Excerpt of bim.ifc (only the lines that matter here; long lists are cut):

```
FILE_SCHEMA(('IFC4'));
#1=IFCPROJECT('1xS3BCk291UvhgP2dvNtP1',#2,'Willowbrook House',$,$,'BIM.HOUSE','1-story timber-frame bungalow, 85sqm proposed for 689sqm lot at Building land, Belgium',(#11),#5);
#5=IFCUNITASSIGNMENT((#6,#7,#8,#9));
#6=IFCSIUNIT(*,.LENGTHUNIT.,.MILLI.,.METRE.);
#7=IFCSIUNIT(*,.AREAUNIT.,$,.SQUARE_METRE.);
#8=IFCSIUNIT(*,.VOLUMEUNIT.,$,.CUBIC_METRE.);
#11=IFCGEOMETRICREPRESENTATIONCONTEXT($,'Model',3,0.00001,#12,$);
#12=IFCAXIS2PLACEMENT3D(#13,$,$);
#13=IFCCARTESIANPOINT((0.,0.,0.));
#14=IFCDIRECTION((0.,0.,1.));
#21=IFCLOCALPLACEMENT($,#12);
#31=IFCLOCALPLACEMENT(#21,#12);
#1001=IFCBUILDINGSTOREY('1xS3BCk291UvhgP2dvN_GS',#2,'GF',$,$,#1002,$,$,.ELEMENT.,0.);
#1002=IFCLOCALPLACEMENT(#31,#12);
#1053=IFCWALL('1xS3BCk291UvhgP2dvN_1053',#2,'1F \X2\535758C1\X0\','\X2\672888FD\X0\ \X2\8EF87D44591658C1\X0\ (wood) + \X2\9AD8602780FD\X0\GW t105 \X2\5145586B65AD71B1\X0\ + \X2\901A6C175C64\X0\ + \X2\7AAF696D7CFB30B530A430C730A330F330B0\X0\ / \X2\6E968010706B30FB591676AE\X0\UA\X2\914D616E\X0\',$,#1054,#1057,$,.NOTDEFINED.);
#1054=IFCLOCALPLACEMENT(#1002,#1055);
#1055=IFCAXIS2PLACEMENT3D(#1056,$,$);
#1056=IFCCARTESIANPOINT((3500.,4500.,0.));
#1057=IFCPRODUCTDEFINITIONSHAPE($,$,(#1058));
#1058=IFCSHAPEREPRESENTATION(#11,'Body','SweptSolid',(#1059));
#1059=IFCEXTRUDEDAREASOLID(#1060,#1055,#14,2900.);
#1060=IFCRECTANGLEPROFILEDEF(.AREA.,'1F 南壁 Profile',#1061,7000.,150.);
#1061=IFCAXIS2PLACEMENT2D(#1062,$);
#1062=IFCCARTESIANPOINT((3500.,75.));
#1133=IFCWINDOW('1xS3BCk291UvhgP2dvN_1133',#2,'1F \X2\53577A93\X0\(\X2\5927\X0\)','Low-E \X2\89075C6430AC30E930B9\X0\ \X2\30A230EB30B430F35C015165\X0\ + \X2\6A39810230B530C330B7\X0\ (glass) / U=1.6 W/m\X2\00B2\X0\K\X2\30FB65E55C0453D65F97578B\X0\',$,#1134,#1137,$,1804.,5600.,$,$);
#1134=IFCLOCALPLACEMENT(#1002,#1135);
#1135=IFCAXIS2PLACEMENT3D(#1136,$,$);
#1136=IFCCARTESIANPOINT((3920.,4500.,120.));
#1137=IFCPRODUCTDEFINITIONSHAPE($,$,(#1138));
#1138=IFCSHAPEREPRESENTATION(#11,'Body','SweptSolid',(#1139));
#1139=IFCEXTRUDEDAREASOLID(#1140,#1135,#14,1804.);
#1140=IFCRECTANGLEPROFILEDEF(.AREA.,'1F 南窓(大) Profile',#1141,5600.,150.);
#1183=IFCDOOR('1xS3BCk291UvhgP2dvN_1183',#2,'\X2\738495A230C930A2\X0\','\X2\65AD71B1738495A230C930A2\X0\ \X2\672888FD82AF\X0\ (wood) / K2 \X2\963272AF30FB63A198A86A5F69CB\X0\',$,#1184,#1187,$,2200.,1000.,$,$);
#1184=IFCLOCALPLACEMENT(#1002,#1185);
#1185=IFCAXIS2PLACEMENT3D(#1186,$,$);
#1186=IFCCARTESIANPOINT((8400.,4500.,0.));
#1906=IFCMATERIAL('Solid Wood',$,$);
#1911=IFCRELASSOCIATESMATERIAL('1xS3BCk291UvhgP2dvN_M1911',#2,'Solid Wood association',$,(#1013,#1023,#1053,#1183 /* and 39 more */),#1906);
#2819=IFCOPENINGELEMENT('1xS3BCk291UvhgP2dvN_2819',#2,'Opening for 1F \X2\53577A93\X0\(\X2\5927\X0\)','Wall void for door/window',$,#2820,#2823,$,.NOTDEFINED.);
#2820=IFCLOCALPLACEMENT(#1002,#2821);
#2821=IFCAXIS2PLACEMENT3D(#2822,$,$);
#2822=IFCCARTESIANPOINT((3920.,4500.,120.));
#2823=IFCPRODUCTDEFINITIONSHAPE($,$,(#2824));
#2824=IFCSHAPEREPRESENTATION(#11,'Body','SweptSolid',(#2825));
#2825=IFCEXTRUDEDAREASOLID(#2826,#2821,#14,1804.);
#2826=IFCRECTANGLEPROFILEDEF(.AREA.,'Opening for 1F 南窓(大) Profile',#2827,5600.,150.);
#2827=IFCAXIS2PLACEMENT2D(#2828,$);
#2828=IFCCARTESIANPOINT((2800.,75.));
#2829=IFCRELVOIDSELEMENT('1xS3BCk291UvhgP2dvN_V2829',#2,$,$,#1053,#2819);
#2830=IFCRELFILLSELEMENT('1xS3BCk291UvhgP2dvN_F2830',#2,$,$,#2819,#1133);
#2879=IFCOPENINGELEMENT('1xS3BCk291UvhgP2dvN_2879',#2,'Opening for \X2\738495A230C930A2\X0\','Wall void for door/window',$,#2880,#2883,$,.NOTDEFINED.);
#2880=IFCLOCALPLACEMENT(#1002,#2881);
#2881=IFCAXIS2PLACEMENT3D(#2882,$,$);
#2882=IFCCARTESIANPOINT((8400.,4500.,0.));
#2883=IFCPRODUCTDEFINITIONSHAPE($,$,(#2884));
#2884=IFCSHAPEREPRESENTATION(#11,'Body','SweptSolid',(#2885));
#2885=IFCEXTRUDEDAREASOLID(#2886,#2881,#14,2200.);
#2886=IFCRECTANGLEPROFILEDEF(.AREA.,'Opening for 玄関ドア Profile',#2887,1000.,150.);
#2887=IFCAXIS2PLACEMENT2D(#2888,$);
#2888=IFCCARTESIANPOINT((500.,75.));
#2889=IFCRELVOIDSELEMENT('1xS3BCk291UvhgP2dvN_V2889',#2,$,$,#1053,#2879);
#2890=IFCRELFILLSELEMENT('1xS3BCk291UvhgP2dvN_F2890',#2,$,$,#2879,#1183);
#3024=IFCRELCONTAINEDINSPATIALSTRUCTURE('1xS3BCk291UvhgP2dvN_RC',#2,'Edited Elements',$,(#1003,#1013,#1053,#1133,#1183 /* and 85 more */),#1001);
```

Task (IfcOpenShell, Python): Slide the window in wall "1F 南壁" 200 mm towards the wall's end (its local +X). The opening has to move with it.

```python
import ifcopenshell
import ifcopenshell.api.geometry
import ifcopenshell.util.placement

model = ifcopenshell.open("bim.ifc")

window = model.by_guid("1xS3BCk291UvhgP2dvN_1133")
opening = window.FillsVoids[0].RelatingOpeningElement
wall = opening.VoidsElements[0].RelatingBuildingElement

wall_matrix = ifcopenshell.util.placement.get_local_placement(wall.ObjectPlacement)
shift = wall_matrix[:3, 0] * 200.0
before = ifcopenshell.util.placement.get_local_placement(window.ObjectPlacement)[:3, 3].copy()

# The window is not placed relative to its opening, so move both.
for product in (opening, window):
    matrix = ifcopenshell.util.placement.get_local_placement(product.ObjectPlacement)
    matrix[:3, 3] += shift
    ifcopenshell.api.geometry.edit_object_placement(model, product=product, matrix=matrix, is_si=False)

after = ifcopenshell.util.placement.get_local_placement(window.ObjectPlacement)[:3, 3]
print("window moved by", (after - before).round(3) + 0.0)

model.write("bim_updated.ifc")
```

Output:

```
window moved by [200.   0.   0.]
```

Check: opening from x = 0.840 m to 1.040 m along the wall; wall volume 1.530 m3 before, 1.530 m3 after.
